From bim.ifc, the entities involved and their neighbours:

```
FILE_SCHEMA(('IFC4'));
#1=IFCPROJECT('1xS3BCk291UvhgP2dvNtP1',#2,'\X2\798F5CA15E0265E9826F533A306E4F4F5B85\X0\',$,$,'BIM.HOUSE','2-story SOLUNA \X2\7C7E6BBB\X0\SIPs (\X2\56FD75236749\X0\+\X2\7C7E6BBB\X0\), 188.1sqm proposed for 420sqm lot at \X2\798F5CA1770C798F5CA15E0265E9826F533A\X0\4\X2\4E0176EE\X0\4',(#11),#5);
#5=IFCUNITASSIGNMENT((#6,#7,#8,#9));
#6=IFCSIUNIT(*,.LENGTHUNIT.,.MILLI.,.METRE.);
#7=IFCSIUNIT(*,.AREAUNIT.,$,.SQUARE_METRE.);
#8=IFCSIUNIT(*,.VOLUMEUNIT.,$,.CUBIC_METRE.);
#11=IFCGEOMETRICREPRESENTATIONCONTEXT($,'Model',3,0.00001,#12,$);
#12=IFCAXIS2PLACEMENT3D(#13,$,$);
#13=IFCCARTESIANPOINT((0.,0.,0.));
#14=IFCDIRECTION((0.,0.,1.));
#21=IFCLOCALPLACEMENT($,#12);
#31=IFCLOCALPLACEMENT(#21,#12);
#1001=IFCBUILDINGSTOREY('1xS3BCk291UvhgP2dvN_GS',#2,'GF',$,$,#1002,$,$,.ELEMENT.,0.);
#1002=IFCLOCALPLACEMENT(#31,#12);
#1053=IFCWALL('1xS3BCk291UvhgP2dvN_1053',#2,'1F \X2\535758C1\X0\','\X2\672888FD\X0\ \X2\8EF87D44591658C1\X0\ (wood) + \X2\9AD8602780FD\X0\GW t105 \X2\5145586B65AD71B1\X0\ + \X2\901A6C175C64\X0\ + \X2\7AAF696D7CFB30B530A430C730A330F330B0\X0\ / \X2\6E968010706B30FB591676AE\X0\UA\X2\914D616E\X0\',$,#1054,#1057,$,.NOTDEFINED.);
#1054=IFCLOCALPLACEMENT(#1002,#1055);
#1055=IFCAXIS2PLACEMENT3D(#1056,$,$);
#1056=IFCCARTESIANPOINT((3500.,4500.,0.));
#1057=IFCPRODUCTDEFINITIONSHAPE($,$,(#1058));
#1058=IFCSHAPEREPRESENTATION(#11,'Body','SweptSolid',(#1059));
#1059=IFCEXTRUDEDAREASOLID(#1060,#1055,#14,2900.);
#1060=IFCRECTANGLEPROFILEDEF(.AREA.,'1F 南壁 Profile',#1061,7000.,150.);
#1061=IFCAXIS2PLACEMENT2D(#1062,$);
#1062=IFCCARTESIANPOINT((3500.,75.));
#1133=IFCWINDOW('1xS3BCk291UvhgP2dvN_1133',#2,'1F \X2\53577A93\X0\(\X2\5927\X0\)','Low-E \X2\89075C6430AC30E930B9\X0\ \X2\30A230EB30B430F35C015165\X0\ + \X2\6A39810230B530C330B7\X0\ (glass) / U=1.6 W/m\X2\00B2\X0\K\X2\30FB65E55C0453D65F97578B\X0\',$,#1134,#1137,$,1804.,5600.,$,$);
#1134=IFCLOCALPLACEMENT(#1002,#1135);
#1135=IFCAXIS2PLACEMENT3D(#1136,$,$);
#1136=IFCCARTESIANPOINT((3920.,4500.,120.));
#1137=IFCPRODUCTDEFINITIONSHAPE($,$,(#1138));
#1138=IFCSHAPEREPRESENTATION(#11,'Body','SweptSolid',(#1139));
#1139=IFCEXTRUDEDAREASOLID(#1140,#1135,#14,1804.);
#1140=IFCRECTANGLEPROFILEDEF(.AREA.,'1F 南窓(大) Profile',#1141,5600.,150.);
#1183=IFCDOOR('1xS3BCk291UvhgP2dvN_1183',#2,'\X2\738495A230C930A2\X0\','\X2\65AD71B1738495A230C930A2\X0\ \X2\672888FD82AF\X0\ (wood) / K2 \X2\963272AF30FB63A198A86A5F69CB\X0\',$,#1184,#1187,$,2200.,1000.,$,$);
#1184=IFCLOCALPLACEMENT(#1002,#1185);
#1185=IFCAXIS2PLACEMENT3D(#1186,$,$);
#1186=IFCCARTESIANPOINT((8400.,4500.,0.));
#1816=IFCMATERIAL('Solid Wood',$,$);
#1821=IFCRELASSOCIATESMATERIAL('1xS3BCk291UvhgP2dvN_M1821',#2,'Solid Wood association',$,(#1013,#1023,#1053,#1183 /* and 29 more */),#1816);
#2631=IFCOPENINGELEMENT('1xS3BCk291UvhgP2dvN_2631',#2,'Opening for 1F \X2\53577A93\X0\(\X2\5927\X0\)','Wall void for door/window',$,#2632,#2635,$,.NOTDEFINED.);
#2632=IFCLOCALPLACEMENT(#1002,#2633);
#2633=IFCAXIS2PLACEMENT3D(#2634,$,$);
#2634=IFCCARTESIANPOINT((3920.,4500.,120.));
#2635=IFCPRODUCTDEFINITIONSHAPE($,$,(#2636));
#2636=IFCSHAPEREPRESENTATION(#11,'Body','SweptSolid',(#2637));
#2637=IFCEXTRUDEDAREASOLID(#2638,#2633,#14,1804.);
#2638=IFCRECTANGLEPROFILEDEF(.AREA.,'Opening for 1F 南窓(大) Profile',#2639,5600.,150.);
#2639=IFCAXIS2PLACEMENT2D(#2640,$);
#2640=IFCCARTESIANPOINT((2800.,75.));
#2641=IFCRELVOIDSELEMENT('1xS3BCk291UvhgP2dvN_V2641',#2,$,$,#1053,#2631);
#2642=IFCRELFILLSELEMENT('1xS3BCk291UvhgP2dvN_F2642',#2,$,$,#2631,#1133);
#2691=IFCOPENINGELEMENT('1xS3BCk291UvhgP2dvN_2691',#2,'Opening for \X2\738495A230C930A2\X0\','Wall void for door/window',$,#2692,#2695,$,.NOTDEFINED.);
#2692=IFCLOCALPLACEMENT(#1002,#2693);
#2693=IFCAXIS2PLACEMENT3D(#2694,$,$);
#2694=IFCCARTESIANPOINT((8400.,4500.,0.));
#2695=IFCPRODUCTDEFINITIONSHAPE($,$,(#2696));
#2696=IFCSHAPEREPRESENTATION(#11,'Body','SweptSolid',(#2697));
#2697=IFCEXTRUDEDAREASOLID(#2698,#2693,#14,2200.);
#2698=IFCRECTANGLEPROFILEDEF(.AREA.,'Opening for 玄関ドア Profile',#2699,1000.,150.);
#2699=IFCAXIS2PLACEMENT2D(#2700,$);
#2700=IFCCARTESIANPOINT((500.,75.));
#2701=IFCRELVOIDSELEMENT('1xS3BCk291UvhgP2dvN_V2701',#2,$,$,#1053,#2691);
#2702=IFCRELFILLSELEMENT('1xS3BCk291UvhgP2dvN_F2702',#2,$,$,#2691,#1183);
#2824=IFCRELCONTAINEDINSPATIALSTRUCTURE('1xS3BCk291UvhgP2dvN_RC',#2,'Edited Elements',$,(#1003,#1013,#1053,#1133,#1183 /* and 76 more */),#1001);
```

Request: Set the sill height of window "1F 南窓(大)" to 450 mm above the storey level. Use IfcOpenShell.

```python
import numpy as np
import ifcopenshell
import ifcopenshell.api.geometry
import ifcopenshell.geom
import ifcopenshell.util.element
import ifcopenshell.util.placement
import ifcopenshell.util.shape
import ifcopenshell.util.unit

model = ifcopenshell.open("bim.ifc")
unit_scale = ifcopenshell.util.unit.calculate_unit_scale(model)

window = model.by_guid("1xS3BCk291UvhgP2dvN_1133")
opening = window.FillsVoids[0].RelatingOpeningElement
storey = ifcopenshell.util.element.get_container(window, ifc_class="IfcBuildingStorey")
level = ifcopenshell.util.placement.get_local_placement(storey.ObjectPlacement)[2, 3]

# The opening's origin need not be at the sill, so measure its lowest point.
shape = ifcopenshell.geom.create_shape(ifcopenshell.geom.settings(), opening)
bottom = ifcopenshell.util.shape.get_shape_bottom_elevation(shape, shape.geometry) / unit_scale
dz = level + 0.45 / unit_scale - bottom

shift = np.array([0.0, 0.0, dz])
# The window is not placed relative to its opening, so move both.
for product in (opening, window):
    matrix = ifcopenshell.util.placement.get_local_placement(product.ObjectPlacement)
    matrix[:3, 3] += shift
    ifcopenshell.api.geometry.edit_object_placement(model, product=product, matrix=matrix, is_si=False)

print(f"moved by {dz * unit_scale:+.3f} m")

model.write("bim_rev.ifc")
```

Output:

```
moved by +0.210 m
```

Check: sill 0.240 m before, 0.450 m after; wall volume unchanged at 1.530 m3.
